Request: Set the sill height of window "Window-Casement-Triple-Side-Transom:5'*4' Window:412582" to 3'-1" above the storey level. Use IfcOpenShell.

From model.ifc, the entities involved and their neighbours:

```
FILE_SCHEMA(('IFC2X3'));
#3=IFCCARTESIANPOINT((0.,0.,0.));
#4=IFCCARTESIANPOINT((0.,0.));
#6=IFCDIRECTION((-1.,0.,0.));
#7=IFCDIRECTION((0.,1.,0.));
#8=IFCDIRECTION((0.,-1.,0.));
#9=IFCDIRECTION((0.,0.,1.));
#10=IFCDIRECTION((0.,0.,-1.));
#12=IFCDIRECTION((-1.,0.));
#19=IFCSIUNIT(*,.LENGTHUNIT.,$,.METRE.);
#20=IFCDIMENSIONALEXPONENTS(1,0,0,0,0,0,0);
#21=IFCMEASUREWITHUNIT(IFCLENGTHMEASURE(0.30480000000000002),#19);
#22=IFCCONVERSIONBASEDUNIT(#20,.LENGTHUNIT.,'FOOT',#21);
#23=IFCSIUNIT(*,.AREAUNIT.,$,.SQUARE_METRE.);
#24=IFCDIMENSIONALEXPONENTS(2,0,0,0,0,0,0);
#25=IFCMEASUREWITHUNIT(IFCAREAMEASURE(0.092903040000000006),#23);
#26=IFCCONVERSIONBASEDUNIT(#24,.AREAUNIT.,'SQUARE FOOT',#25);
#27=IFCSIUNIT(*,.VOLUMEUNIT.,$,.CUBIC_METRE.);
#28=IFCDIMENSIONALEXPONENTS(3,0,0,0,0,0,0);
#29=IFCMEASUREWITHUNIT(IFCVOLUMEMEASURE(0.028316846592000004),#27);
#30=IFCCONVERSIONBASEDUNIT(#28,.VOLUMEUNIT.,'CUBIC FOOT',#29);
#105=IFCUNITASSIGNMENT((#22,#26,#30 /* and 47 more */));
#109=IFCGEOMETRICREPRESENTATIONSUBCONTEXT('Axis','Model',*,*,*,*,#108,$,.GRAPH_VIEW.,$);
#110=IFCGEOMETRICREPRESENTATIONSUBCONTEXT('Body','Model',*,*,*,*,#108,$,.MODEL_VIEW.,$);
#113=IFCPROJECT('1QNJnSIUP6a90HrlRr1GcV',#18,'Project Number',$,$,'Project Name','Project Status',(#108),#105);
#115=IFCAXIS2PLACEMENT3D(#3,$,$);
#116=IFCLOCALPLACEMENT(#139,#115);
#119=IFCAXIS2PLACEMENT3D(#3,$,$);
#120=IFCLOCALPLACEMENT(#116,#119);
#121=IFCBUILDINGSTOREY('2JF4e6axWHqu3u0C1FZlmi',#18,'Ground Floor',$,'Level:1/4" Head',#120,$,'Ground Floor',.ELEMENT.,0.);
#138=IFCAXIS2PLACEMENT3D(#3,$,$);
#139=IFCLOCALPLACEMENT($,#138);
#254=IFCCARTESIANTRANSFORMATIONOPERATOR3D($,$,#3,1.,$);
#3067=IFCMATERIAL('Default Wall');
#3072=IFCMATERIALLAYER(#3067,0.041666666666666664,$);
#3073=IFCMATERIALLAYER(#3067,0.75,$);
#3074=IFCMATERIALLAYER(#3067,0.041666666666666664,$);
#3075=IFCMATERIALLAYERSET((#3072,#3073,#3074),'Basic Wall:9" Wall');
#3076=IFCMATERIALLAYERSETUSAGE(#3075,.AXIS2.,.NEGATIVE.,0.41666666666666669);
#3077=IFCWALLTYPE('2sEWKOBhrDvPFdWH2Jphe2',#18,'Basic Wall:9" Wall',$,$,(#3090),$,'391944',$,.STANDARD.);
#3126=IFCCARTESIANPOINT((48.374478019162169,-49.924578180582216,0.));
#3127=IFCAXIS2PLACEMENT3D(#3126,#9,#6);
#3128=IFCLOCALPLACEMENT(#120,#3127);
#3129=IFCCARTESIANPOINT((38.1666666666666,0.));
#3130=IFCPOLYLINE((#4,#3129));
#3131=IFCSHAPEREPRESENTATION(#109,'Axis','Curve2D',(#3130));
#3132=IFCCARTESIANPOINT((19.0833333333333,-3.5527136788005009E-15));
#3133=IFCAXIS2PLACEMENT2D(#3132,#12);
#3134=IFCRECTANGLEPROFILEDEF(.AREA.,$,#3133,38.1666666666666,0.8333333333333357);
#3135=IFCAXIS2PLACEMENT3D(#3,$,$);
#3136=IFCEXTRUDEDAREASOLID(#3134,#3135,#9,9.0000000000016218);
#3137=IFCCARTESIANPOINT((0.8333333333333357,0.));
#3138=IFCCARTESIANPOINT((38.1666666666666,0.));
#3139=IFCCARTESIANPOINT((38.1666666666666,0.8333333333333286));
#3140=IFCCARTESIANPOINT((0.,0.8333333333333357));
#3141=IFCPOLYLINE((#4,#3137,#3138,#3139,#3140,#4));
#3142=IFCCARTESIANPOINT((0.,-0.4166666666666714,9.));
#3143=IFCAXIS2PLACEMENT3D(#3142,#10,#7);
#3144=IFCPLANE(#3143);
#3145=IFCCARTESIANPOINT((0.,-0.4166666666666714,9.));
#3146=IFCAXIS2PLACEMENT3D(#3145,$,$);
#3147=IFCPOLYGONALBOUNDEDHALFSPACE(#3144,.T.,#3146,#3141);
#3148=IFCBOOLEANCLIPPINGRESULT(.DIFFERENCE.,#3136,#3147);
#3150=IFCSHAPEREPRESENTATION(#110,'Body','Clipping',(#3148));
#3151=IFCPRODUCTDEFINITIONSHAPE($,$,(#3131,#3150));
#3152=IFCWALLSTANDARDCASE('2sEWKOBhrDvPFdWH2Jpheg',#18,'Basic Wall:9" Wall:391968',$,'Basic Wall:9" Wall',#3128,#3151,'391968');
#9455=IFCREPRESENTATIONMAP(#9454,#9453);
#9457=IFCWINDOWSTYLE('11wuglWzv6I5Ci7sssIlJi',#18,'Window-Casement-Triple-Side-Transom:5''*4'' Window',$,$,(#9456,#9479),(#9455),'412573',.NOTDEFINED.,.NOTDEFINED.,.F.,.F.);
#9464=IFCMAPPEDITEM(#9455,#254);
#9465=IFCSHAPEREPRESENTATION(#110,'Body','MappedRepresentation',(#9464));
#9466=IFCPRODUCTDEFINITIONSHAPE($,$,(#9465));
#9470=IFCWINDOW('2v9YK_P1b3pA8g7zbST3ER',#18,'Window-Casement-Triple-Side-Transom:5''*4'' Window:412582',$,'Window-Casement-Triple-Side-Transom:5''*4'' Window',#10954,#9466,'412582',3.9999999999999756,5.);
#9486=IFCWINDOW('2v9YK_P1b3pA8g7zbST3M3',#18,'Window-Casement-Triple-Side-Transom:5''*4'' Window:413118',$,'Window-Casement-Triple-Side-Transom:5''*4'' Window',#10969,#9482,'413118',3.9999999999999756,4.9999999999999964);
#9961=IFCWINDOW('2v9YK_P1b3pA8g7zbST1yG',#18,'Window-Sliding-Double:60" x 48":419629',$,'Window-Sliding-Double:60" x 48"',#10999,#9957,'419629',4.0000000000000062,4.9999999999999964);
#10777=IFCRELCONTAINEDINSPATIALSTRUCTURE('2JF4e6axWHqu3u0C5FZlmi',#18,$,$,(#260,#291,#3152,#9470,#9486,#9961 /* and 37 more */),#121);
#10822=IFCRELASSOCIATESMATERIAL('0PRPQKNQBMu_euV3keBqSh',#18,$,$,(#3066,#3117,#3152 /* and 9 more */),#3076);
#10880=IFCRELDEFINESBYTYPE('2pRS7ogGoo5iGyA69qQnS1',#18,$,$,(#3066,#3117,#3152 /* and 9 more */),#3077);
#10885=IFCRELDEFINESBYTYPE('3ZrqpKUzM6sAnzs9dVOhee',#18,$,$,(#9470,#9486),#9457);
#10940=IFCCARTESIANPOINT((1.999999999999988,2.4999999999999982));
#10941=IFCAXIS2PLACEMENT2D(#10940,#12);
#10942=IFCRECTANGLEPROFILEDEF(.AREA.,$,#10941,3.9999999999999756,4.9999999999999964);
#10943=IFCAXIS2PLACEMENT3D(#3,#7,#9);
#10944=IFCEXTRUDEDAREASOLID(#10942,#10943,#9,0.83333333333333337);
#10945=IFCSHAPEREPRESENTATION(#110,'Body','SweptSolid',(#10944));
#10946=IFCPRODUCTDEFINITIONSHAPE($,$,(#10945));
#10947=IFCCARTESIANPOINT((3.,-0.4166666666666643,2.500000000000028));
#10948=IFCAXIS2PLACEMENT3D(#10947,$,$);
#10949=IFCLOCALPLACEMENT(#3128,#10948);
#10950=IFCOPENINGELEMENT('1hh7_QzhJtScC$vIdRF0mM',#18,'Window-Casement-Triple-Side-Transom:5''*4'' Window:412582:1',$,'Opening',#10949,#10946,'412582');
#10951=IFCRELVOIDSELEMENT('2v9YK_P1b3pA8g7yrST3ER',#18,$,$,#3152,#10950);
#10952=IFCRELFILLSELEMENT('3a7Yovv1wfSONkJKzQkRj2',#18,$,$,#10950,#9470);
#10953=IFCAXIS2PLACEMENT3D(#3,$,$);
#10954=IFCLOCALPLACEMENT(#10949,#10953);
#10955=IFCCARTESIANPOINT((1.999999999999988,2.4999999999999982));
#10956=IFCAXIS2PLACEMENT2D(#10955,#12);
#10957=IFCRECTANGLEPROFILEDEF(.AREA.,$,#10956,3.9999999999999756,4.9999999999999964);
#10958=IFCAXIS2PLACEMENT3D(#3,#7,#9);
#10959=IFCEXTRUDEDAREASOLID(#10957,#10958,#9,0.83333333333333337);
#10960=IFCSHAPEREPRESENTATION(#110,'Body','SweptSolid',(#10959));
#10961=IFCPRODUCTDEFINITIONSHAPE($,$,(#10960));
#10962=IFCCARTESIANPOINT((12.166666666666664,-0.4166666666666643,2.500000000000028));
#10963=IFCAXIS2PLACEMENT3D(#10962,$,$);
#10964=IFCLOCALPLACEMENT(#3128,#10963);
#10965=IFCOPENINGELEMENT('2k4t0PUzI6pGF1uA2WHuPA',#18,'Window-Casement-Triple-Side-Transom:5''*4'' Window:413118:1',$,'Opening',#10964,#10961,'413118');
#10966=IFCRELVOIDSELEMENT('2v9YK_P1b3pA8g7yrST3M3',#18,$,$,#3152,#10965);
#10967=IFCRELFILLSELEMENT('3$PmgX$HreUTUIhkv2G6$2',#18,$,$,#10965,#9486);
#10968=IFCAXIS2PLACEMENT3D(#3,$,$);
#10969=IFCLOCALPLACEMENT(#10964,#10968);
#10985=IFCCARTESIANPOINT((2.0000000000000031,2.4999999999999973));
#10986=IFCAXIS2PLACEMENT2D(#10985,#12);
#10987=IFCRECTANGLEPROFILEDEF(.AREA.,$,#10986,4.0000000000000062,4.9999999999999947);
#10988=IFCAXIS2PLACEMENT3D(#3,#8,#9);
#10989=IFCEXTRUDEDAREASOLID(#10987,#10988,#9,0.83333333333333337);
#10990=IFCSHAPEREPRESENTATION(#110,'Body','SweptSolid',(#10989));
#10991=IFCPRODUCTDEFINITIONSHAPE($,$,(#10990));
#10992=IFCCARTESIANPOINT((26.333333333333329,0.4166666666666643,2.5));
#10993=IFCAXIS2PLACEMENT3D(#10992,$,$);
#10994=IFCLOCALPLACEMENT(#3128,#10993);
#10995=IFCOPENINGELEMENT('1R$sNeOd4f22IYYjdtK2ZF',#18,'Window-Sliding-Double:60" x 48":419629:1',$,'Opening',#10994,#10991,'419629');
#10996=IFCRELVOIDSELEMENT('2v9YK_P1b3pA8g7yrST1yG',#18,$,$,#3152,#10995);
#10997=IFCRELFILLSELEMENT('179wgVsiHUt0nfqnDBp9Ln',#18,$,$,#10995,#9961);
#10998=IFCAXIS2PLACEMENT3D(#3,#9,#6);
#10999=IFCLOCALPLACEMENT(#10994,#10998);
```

```python
import numpy as np
import ifcopenshell
import ifcopenshell.api.geometry
import ifcopenshell.geom
import ifcopenshell.util.element
import ifcopenshell.util.placement
import ifcopenshell.util.shape
import ifcopenshell.util.unit

model = ifcopenshell.open("model.ifc")
unit_scale = ifcopenshell.util.unit.calculate_unit_scale(model)

window = model.by_guid("2v9YK_P1b3pA8g7zbST3ER")
opening = window.FillsVoids[0].RelatingOpeningElement
storey = ifcopenshell.util.element.get_container(window, ifc_class="IfcBuildingStorey")
level = ifcopenshell.util.placement.get_local_placement(storey.ObjectPlacement)[2, 3]

# The opening's origin need not be at the sill, so measure its lowest point.
shape = ifcopenshell.geom.create_shape(ifcopenshell.geom.settings(), opening)
bottom = ifcopenshell.util.shape.get_shape_bottom_elevation(shape, shape.geometry) / unit_scale
dz = level + 37 * 0.0254 / unit_scale - bottom

shift = np.array([0.0, 0.0, dz])
# The window is placed relative to its opening, so it follows when the opening moves.
matrix = ifcopenshell.util.placement.get_local_placement(opening.ObjectPlacement)
matrix[:3, 3] += shift
ifcopenshell.api.geometry.edit_object_placement(
    model, product=opening, matrix=matrix, is_si=False, should_transform_children=True
)

print(f"moved by {dz * unit_scale:+.3f} m")

model.write("model-out.ifc")
```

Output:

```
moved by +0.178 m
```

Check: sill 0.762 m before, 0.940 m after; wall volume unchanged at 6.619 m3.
